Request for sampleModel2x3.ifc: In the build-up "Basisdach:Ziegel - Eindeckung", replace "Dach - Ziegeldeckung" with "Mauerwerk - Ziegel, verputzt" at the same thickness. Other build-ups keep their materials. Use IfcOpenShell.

First a look at what the model holds.

```python
import ifcopenshell
import ifcopenshell.util.element

model = ifcopenshell.open("sampleModel2x3.ifc")
print(model.schema)
for layer_set in model.by_type("IfcMaterialLayerSet"):
    if layer_set.LayerSetName == "Basisdach:Ziegel - Eindeckung":
        for layer in layer_set.MaterialLayers:
            print(layer.id(), layer.Material and layer.Material.Name, layer.LayerThickness, sep=" | ")
        print(len(ifcopenshell.util.element.get_elements_by_material(model, layer_set)), "elements and types use it")
print(sorted(m.Name for m in model.by_type("IfcMaterial") if m.Name)[:60])
```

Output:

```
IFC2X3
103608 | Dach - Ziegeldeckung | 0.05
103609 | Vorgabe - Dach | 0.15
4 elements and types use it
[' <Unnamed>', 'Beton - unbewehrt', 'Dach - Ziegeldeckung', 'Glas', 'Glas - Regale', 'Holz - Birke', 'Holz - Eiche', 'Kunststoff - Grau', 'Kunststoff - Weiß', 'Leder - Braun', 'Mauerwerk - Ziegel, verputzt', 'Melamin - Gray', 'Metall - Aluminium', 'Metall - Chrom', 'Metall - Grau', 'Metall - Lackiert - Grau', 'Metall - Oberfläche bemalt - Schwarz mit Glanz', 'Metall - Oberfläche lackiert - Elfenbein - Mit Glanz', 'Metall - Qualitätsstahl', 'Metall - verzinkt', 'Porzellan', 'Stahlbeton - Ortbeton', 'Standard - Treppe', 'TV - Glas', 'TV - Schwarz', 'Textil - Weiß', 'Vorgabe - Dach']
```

```python
import ifcopenshell
import ifcopenshell.api.material

model = ifcopenshell.open("sampleModel2x3.ifc")

layer_set = next(s for s in model.by_type("IfcMaterialLayerSet") if s.LayerSetName == "Basisdach:Ziegel - Eindeckung")
layer = next(l for l in layer_set.MaterialLayers if l.Material and l.Material.Name == "Dach - Ziegeldeckung")
material = next(m for m in model.by_type("IfcMaterial") if m.Name == "Mauerwerk - Ziegel, verputzt")

# Point this one layer at the other material; renaming the old one would change it everywhere.
ifcopenshell.api.material.edit_layer(model, layer=layer, attributes={}, material=material)

print([l.Material.Name if l.Material else None for l in layer_set.MaterialLayers])

model.write("sampleModel2x3-out.ifc")
```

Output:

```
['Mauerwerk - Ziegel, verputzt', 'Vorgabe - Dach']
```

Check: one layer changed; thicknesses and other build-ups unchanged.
